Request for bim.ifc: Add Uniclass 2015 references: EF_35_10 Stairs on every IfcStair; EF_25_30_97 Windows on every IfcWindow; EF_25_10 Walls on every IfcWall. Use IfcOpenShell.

First a look at what the model holds.

```python
import ifcopenshell

model = ifcopenshell.open("bim.ifc")
print(model.schema)
print("classifications:", [c.Name for c in model.by_type("IfcClassification")])
for ifc_class in ("IfcDoor", "IfcRoof", "IfcStair", "IfcWall", "IfcWindow"):
    print(ifc_class, len(model.by_type(ifc_class)))
```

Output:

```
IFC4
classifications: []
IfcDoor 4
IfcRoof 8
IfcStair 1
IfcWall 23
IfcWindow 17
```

```python
import ifcopenshell
import ifcopenshell.api.classification

model = ifcopenshell.open("bim.ifc")

system = ifcopenshell.api.classification.add_classification(model, classification="Uniclass 2015")

codes = {
    "IfcStair": ("EF_35_10", "Stairs"),
    "IfcWindow": ("EF_25_30_97", "Windows"),
    "IfcWall": ("EF_25_10", "Walls"),
}
for ifc_class, (code, name) in codes.items():
    products = model.by_type(ifc_class)
    ifcopenshell.api.classification.add_reference(
        model, products=products, classification=system, identification=code, name=name
    )
    print(code, len(products))

model.write("bim_rev.ifc")
```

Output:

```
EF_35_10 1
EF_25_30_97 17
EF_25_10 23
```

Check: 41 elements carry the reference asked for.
